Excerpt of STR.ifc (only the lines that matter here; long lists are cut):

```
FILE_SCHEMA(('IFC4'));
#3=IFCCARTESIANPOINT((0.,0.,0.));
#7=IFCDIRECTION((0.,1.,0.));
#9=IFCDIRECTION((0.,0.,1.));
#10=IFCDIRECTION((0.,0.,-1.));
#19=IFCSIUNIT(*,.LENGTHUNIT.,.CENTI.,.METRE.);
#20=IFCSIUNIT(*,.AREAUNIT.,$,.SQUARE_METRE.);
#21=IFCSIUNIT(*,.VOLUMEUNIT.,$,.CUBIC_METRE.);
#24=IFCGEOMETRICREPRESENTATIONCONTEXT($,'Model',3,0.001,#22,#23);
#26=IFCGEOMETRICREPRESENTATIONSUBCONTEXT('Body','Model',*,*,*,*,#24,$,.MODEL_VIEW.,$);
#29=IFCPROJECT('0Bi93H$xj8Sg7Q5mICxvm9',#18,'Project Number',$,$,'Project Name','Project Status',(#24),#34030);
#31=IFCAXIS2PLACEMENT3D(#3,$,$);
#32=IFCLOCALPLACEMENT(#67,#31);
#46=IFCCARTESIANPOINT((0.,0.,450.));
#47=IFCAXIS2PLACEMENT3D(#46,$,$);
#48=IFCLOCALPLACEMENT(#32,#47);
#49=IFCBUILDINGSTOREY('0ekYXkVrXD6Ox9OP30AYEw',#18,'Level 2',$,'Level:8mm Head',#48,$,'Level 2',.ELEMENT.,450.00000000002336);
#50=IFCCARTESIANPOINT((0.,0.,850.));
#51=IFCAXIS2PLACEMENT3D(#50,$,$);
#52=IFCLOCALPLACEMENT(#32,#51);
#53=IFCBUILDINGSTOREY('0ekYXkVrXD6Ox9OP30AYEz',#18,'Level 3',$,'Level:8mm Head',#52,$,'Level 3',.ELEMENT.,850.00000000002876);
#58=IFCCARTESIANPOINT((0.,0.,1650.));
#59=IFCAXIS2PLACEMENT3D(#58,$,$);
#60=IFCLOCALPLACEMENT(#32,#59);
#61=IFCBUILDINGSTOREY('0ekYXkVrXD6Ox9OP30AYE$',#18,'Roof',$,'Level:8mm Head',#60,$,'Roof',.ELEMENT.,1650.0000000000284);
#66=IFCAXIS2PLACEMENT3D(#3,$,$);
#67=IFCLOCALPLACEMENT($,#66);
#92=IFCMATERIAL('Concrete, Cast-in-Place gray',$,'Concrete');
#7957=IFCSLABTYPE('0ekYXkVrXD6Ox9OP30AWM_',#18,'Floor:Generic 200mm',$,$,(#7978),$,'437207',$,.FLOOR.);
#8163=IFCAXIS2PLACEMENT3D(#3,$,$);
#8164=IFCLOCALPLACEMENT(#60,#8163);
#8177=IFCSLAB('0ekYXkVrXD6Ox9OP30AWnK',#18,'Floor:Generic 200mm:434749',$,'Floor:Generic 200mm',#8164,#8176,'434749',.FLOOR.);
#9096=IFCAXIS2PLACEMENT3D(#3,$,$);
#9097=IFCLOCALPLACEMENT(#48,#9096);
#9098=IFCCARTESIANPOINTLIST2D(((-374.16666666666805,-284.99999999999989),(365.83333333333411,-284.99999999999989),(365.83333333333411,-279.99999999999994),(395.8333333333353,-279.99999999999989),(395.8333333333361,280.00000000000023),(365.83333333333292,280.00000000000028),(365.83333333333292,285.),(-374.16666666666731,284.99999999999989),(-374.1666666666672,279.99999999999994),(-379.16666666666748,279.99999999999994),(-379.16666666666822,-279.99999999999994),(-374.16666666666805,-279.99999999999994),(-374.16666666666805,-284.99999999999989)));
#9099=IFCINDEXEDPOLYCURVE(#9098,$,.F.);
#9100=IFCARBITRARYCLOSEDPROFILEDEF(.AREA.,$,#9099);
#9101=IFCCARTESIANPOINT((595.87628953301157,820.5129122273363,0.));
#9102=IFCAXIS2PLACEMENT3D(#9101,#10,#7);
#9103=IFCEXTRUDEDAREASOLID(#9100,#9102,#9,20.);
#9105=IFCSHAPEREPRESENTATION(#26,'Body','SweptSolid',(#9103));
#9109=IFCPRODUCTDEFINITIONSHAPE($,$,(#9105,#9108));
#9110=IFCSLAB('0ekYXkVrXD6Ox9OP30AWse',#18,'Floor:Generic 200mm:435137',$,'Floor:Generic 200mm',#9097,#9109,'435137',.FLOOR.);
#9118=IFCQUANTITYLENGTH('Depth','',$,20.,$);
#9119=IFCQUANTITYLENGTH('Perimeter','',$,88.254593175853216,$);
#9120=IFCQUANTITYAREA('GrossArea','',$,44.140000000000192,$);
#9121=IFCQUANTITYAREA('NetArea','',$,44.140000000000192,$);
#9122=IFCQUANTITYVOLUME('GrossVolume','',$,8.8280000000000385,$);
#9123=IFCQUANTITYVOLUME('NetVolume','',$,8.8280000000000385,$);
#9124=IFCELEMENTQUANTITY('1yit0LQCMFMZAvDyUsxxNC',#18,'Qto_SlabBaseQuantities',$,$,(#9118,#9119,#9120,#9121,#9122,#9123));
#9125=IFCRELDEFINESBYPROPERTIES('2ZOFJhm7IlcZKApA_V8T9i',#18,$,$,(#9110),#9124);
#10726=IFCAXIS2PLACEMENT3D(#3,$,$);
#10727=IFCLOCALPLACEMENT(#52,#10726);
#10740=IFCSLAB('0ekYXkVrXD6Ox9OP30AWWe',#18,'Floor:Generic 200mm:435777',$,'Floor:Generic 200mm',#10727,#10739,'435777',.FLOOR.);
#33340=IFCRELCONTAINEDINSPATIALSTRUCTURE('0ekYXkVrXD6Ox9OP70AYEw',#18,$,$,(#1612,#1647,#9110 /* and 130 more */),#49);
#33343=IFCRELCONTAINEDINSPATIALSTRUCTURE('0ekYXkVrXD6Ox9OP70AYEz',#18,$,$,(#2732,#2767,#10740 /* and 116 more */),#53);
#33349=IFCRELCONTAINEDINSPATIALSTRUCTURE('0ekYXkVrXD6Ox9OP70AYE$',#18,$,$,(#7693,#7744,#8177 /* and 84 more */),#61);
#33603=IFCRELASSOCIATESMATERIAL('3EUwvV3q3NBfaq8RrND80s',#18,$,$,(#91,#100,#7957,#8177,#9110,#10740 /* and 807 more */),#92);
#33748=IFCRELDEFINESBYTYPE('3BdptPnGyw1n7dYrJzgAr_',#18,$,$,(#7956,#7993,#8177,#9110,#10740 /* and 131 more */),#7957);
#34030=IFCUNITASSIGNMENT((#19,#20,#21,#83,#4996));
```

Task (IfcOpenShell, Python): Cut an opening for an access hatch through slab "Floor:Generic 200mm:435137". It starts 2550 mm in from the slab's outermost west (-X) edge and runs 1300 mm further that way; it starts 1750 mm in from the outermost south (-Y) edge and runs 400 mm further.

```python
import numpy as np
import ifcopenshell
import ifcopenshell.api.feature
import ifcopenshell.api.geometry
import ifcopenshell.api.pset
import ifcopenshell.api.root
import ifcopenshell.geom
import ifcopenshell.util.element
import ifcopenshell.util.placement
import ifcopenshell.util.representation
import ifcopenshell.util.shape
import ifcopenshell.util.unit

model = ifcopenshell.open("STR.ifc")
unit_scale = ifcopenshell.util.unit.calculate_unit_scale(model)
area_scale = ifcopenshell.util.unit.calculate_unit_scale(model, "AREAUNIT")
volume_scale = ifcopenshell.util.unit.calculate_unit_scale(model, "VOLUMEUNIT")
settings = ifcopenshell.geom.settings()


def volume(element):
    """Net volume in cubic metres, openings subtracted."""
    shape = ifcopenshell.geom.create_shape(settings, element)
    return ifcopenshell.util.shape.get_volume(shape.geometry)


slab = model.by_guid("0ekYXkVrXD6Ox9OP30AWse")
before = volume(slab)

# Extent in the slab's own axes, in metres. The edges named are its -X and -Y sides.
slab_shape = ifcopenshell.geom.create_shape(settings, slab)
vertices = ifcopenshell.util.shape.get_vertices(slab_shape.geometry)
x_min, y_min, bottom = vertices.min(axis=0)
top = vertices[:, 2].max()

opening = ifcopenshell.api.root.create_entity(model, ifc_class="IfcOpeningElement", name="Access hatch opening", predefined_type="OPENING")
context = ifcopenshell.util.representation.get_context(model, "Model", "Body", "MODEL_VIEW")
width, depth = 1.3, 0.4
outline = [(0.0, 0.0), (width, 0.0), (width, depth), (0.0, depth), (0.0, 0.0)]
# Overshoot both faces by 50 mm so the cut is clean.
shape = ifcopenshell.api.geometry.add_slab_representation(
    model, context=context, depth=top - bottom + 0.1, polyline=outline
)
ifcopenshell.api.geometry.assign_representation(model, product=opening, representation=shape)

matrix = ifcopenshell.util.placement.get_local_placement(slab.ObjectPlacement)
matrix[:, 3] = matrix @ np.append(np.array([x_min + 2.55, y_min + 1.75, bottom - 0.05]) / unit_scale, 1.0)
ifcopenshell.api.geometry.edit_object_placement(model, product=opening, matrix=matrix, is_si=False)
ifcopenshell.api.feature.add_feature(model, feature=opening, element=slab)

after = volume(slab)

# Update the slab's stored quantities.
qto = model.by_id(ifcopenshell.util.element.get_pset(slab, "Qto_SlabBaseQuantities", should_inherit=False)["id"])
ifcopenshell.api.pset.edit_qto(model, qto=qto, properties={
    "NetArea": after / (top - bottom) / area_scale,
    "NetVolume": after / volume_scale,
})

print(f"slab volume {before:.3f} -> {after:.3f} m3")

model.write("STR_v2.ifc")
```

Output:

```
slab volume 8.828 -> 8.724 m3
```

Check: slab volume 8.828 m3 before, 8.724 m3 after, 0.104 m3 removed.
